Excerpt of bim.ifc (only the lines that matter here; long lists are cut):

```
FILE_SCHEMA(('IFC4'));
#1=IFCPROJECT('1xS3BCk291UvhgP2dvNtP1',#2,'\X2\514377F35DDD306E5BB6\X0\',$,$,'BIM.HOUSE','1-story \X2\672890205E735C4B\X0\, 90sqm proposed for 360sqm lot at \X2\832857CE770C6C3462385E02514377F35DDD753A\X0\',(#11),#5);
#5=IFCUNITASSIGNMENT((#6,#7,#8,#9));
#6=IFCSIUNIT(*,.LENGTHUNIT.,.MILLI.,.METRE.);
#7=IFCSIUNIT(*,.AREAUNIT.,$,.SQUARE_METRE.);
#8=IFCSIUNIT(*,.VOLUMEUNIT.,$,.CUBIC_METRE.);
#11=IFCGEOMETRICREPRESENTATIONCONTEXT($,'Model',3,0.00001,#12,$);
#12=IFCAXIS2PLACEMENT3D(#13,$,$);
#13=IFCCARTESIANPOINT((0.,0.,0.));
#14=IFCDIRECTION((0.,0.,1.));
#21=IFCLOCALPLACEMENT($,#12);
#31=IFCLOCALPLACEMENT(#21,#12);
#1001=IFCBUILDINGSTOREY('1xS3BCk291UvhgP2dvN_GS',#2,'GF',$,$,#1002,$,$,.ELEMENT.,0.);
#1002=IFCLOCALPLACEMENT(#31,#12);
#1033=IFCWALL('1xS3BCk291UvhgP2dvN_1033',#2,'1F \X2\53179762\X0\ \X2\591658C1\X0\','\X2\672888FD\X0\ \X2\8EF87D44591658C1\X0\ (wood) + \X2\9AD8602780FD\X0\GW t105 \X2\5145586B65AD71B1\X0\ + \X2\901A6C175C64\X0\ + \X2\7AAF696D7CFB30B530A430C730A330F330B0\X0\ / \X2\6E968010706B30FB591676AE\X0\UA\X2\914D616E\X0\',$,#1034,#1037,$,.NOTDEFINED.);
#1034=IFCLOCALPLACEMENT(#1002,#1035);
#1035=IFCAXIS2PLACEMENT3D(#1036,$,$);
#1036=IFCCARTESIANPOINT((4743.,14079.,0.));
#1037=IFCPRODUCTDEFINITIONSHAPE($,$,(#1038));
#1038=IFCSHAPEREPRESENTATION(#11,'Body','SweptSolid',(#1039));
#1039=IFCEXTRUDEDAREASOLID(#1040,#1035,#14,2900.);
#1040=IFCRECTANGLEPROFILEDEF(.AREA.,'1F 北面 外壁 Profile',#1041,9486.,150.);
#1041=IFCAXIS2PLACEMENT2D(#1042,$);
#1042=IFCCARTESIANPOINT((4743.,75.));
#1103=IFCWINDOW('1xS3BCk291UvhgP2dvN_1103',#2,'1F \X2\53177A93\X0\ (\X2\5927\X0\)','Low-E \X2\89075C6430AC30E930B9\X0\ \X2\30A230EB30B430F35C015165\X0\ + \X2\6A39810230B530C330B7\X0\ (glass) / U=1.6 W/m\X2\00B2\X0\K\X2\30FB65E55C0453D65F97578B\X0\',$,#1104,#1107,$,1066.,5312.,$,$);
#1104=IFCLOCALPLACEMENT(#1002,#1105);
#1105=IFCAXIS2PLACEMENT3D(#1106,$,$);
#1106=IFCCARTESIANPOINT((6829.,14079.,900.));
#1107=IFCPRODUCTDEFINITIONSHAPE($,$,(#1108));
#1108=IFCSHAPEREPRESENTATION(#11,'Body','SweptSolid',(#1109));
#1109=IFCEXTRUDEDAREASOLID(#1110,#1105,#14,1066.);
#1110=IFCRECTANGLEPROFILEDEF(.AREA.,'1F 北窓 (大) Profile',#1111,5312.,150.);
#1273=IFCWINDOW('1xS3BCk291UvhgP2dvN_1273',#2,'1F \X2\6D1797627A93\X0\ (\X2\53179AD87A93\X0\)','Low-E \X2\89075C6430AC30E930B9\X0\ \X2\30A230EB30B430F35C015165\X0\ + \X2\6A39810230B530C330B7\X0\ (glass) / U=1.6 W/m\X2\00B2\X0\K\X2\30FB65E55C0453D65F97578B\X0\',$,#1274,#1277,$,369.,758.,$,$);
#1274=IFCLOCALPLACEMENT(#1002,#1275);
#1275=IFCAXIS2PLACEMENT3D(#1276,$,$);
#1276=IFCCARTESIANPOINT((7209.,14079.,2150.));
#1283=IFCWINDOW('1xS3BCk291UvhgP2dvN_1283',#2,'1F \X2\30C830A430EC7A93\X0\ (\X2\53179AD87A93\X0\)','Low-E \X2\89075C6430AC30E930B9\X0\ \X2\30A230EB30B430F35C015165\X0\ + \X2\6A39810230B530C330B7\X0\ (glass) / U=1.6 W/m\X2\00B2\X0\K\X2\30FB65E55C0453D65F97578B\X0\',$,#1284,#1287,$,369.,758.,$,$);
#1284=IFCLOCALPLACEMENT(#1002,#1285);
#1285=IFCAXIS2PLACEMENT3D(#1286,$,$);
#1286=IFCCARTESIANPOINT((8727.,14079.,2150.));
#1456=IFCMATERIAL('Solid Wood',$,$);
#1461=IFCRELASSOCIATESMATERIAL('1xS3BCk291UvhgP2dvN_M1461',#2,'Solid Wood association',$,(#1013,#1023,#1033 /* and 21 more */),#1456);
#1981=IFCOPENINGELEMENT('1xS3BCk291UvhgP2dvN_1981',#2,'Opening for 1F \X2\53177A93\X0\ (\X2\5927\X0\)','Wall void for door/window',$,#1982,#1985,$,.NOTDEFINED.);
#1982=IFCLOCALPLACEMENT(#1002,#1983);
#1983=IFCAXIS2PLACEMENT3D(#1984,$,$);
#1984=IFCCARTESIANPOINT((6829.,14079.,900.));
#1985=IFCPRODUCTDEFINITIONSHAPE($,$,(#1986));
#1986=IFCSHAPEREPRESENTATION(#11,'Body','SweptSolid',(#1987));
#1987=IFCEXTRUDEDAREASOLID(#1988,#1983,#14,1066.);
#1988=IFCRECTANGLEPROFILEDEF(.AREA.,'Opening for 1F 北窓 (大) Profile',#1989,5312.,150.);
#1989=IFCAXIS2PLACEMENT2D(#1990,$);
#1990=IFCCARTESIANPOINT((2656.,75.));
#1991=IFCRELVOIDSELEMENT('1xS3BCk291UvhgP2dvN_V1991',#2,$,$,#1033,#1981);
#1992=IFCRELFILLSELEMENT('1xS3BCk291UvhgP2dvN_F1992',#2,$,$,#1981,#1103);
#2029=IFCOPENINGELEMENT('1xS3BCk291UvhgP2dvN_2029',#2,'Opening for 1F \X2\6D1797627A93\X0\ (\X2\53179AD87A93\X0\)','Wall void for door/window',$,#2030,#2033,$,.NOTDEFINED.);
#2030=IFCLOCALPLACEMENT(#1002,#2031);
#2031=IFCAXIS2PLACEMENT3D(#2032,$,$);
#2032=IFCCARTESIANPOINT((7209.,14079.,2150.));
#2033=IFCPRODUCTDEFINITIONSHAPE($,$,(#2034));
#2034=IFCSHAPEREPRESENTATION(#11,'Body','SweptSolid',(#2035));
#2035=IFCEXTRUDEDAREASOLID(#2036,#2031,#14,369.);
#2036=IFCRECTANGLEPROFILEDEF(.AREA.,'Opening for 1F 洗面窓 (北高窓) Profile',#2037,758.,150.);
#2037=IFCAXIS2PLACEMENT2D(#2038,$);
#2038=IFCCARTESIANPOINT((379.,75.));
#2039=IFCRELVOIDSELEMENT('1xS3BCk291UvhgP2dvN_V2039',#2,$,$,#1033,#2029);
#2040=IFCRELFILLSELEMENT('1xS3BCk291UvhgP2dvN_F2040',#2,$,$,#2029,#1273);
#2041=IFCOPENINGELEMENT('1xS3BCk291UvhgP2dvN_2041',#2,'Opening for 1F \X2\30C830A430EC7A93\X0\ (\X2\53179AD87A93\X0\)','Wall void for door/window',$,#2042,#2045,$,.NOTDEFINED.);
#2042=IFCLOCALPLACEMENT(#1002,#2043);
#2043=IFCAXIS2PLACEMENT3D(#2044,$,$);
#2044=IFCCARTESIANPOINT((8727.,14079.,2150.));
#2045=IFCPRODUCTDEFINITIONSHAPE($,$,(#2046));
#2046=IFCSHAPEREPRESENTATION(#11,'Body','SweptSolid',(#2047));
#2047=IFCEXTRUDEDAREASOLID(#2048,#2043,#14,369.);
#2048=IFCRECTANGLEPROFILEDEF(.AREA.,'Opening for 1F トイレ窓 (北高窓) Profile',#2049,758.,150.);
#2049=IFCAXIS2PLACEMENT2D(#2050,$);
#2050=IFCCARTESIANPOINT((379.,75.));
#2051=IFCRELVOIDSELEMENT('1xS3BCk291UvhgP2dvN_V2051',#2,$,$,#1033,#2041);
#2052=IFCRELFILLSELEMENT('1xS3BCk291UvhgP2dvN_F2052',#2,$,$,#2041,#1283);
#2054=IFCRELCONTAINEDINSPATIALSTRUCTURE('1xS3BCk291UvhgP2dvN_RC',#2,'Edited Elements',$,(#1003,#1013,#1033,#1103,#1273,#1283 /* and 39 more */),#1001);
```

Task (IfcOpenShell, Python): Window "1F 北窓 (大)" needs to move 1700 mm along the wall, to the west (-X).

```python
import ifcopenshell
import ifcopenshell.api.geometry
import ifcopenshell.util.placement

model = ifcopenshell.open("bim.ifc")

window = model.by_guid("1xS3BCk291UvhgP2dvN_1103")
opening = window.FillsVoids[0].RelatingOpeningElement
wall = opening.VoidsElements[0].RelatingBuildingElement

wall_matrix = ifcopenshell.util.placement.get_local_placement(wall.ObjectPlacement)
shift = wall_matrix[:3, 0] * -1700.0
before = ifcopenshell.util.placement.get_local_placement(window.ObjectPlacement)[:3, 3].copy()

# The window is not placed relative to its opening, so move both.
for product in (opening, window):
    matrix = ifcopenshell.util.placement.get_local_placement(product.ObjectPlacement)
    matrix[:3, 3] += shift
    ifcopenshell.api.geometry.edit_object_placement(model, product=product, matrix=matrix, is_si=False)

after = ifcopenshell.util.placement.get_local_placement(window.ObjectPlacement)[:3, 3]
print("window moved by", (after - before).round(3) + 0.0)

model.write("bim_updated.ifc")
```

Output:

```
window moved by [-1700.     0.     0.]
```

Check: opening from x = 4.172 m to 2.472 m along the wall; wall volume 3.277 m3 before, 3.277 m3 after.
